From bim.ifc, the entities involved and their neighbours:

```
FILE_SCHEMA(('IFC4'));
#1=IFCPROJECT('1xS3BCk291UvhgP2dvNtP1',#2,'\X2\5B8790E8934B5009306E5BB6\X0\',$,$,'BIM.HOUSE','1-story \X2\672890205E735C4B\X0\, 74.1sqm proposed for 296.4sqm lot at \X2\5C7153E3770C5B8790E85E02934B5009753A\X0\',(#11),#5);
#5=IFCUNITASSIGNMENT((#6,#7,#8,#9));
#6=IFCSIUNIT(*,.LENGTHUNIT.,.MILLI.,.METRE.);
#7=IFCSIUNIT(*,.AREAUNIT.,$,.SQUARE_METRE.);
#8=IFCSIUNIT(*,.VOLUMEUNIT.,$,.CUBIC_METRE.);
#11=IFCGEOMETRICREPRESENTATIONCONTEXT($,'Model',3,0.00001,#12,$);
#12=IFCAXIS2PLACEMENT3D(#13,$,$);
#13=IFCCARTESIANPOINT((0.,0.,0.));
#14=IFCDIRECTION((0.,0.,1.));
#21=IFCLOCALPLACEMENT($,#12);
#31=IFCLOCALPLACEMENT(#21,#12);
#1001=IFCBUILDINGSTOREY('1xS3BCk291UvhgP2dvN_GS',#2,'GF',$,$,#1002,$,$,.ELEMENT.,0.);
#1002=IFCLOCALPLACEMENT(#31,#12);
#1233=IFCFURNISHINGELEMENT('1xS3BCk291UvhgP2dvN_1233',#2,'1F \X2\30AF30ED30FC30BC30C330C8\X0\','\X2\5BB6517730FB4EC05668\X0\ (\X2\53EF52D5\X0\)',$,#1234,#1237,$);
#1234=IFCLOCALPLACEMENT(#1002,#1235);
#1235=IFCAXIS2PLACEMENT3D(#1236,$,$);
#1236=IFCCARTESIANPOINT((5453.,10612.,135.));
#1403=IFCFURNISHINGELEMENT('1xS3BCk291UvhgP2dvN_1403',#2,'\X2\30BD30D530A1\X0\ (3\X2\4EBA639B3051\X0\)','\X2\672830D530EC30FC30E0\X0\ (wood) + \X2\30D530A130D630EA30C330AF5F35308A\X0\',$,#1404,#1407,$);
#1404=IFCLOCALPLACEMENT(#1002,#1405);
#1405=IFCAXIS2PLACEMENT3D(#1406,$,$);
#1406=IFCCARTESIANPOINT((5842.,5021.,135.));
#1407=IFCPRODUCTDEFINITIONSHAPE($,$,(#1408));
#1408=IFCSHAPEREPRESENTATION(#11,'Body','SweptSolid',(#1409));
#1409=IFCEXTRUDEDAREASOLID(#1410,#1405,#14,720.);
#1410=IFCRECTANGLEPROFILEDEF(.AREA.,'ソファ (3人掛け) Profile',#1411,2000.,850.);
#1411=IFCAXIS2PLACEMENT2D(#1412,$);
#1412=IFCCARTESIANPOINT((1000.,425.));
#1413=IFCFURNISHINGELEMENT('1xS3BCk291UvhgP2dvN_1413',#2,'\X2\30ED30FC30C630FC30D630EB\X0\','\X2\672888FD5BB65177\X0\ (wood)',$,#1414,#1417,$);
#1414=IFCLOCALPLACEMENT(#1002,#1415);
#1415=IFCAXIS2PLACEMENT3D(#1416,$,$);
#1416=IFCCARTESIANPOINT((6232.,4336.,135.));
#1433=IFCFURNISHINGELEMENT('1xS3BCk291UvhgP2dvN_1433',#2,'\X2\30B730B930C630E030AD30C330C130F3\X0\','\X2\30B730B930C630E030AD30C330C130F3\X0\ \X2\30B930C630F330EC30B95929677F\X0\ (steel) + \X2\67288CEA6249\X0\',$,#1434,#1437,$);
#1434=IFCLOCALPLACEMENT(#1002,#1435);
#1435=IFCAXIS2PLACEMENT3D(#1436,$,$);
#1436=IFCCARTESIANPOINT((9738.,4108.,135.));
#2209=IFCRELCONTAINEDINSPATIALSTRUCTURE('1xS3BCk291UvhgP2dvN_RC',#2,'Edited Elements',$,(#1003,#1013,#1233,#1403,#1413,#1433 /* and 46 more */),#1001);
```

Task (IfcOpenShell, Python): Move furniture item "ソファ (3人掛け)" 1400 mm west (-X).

```python
import ifcopenshell
import ifcopenshell.api.geometry
import ifcopenshell.util.placement
import ifcopenshell.util.unit

model = ifcopenshell.open("bim.ifc")
unit_scale = ifcopenshell.util.unit.calculate_unit_scale(model)

item = model.by_guid("1xS3BCk291UvhgP2dvN_1403")
matrix = ifcopenshell.util.placement.get_local_placement(item.ObjectPlacement)
matrix[0, 3] -= 1.4 / unit_scale
ifcopenshell.api.geometry.edit_object_placement(model, product=item, matrix=matrix, is_si=False)

print(ifcopenshell.util.placement.get_local_placement(item.ObjectPlacement).round(3) + 0.0)

model.write("bim-out.ifc")
```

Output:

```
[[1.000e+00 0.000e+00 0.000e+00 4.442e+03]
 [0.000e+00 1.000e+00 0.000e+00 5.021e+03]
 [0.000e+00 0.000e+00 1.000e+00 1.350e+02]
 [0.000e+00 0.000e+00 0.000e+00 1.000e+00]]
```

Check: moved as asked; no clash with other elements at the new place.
